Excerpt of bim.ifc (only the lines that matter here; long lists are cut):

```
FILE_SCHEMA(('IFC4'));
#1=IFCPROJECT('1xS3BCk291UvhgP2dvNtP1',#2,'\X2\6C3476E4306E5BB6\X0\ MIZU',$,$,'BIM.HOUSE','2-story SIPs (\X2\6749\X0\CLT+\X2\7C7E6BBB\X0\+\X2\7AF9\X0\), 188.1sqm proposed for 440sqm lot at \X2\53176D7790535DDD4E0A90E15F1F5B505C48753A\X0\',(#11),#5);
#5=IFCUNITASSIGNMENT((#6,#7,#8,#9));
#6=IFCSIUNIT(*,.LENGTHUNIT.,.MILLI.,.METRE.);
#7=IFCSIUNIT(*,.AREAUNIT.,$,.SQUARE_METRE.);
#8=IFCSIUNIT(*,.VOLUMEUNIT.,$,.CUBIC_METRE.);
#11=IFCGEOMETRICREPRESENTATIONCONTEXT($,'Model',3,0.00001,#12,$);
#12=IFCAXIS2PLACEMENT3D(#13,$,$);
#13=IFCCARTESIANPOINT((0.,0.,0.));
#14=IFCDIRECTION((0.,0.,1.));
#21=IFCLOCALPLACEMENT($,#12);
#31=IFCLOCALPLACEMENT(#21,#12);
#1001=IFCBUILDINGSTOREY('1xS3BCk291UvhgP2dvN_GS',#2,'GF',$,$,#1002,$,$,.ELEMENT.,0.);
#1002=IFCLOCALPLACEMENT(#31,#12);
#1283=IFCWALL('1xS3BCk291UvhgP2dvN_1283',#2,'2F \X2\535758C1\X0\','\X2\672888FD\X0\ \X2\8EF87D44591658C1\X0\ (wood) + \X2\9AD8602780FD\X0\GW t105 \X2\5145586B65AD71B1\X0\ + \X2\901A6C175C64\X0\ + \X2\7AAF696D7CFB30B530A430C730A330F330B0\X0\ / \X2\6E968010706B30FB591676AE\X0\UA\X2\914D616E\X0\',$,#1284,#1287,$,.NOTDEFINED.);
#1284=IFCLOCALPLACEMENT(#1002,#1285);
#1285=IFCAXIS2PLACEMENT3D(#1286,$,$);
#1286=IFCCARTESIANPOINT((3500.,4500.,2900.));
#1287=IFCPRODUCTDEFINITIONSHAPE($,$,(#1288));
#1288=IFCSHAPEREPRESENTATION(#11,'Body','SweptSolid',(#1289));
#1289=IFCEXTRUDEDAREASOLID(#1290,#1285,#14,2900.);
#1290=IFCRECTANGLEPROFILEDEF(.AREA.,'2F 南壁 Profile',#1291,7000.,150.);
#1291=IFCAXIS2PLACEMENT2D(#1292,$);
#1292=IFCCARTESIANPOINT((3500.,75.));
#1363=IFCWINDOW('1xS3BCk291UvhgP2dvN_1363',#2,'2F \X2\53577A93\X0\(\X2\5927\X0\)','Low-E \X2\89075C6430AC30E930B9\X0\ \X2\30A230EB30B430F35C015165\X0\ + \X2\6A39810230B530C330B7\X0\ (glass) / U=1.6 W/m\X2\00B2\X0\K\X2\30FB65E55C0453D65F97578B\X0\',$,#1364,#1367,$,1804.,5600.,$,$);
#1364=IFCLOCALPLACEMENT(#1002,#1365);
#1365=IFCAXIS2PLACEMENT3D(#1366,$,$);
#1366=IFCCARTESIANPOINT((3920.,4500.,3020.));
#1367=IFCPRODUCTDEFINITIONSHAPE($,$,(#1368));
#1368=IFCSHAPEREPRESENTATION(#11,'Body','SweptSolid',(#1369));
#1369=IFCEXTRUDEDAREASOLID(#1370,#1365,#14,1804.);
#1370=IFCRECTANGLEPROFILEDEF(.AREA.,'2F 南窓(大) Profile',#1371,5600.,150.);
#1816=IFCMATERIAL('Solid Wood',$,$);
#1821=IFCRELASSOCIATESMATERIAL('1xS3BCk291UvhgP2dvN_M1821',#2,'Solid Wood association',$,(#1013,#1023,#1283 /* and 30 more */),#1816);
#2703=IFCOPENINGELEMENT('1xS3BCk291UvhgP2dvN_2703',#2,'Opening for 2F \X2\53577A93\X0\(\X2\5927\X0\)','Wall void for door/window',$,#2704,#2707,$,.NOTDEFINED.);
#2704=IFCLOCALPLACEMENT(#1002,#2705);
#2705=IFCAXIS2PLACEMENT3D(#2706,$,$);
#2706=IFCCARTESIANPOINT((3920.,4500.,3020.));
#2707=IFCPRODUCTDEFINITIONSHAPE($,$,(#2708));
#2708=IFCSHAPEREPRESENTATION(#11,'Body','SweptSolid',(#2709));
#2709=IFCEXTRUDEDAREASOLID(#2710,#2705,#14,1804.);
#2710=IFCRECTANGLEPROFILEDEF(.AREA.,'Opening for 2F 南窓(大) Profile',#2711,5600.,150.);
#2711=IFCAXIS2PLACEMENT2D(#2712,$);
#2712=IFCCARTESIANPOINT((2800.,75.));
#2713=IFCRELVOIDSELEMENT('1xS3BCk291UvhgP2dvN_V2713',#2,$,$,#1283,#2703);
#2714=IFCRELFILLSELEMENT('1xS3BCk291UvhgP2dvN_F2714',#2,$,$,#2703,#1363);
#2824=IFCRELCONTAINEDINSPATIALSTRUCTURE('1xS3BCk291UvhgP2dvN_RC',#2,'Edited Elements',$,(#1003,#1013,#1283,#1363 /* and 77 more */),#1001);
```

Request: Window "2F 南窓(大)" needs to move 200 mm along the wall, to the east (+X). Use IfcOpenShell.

```python
import ifcopenshell
import ifcopenshell.api.geometry
import ifcopenshell.util.placement

model = ifcopenshell.open("bim.ifc")

window = model.by_id(1363)
opening = window.FillsVoids[0].RelatingOpeningElement
wall = opening.VoidsElements[0].RelatingBuildingElement

wall_matrix = ifcopenshell.util.placement.get_local_placement(wall.ObjectPlacement)
shift = wall_matrix[:3, 0] * 200.0
before = ifcopenshell.util.placement.get_local_placement(window.ObjectPlacement)[:3, 3].copy()

# The window is not placed relative to its opening, so move both.
for product in (opening, window):
    matrix = ifcopenshell.util.placement.get_local_placement(product.ObjectPlacement)
    matrix[:3, 3] += shift
    ifcopenshell.api.geometry.edit_object_placement(model, product=product, matrix=matrix, is_si=False)

after = ifcopenshell.util.placement.get_local_placement(window.ObjectPlacement)[:3, 3]
print("window moved by", (after - before).round(3) + 0.0)

model.write("bim_edited.ifc")
```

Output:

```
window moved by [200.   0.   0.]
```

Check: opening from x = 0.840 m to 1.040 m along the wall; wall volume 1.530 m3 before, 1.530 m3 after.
